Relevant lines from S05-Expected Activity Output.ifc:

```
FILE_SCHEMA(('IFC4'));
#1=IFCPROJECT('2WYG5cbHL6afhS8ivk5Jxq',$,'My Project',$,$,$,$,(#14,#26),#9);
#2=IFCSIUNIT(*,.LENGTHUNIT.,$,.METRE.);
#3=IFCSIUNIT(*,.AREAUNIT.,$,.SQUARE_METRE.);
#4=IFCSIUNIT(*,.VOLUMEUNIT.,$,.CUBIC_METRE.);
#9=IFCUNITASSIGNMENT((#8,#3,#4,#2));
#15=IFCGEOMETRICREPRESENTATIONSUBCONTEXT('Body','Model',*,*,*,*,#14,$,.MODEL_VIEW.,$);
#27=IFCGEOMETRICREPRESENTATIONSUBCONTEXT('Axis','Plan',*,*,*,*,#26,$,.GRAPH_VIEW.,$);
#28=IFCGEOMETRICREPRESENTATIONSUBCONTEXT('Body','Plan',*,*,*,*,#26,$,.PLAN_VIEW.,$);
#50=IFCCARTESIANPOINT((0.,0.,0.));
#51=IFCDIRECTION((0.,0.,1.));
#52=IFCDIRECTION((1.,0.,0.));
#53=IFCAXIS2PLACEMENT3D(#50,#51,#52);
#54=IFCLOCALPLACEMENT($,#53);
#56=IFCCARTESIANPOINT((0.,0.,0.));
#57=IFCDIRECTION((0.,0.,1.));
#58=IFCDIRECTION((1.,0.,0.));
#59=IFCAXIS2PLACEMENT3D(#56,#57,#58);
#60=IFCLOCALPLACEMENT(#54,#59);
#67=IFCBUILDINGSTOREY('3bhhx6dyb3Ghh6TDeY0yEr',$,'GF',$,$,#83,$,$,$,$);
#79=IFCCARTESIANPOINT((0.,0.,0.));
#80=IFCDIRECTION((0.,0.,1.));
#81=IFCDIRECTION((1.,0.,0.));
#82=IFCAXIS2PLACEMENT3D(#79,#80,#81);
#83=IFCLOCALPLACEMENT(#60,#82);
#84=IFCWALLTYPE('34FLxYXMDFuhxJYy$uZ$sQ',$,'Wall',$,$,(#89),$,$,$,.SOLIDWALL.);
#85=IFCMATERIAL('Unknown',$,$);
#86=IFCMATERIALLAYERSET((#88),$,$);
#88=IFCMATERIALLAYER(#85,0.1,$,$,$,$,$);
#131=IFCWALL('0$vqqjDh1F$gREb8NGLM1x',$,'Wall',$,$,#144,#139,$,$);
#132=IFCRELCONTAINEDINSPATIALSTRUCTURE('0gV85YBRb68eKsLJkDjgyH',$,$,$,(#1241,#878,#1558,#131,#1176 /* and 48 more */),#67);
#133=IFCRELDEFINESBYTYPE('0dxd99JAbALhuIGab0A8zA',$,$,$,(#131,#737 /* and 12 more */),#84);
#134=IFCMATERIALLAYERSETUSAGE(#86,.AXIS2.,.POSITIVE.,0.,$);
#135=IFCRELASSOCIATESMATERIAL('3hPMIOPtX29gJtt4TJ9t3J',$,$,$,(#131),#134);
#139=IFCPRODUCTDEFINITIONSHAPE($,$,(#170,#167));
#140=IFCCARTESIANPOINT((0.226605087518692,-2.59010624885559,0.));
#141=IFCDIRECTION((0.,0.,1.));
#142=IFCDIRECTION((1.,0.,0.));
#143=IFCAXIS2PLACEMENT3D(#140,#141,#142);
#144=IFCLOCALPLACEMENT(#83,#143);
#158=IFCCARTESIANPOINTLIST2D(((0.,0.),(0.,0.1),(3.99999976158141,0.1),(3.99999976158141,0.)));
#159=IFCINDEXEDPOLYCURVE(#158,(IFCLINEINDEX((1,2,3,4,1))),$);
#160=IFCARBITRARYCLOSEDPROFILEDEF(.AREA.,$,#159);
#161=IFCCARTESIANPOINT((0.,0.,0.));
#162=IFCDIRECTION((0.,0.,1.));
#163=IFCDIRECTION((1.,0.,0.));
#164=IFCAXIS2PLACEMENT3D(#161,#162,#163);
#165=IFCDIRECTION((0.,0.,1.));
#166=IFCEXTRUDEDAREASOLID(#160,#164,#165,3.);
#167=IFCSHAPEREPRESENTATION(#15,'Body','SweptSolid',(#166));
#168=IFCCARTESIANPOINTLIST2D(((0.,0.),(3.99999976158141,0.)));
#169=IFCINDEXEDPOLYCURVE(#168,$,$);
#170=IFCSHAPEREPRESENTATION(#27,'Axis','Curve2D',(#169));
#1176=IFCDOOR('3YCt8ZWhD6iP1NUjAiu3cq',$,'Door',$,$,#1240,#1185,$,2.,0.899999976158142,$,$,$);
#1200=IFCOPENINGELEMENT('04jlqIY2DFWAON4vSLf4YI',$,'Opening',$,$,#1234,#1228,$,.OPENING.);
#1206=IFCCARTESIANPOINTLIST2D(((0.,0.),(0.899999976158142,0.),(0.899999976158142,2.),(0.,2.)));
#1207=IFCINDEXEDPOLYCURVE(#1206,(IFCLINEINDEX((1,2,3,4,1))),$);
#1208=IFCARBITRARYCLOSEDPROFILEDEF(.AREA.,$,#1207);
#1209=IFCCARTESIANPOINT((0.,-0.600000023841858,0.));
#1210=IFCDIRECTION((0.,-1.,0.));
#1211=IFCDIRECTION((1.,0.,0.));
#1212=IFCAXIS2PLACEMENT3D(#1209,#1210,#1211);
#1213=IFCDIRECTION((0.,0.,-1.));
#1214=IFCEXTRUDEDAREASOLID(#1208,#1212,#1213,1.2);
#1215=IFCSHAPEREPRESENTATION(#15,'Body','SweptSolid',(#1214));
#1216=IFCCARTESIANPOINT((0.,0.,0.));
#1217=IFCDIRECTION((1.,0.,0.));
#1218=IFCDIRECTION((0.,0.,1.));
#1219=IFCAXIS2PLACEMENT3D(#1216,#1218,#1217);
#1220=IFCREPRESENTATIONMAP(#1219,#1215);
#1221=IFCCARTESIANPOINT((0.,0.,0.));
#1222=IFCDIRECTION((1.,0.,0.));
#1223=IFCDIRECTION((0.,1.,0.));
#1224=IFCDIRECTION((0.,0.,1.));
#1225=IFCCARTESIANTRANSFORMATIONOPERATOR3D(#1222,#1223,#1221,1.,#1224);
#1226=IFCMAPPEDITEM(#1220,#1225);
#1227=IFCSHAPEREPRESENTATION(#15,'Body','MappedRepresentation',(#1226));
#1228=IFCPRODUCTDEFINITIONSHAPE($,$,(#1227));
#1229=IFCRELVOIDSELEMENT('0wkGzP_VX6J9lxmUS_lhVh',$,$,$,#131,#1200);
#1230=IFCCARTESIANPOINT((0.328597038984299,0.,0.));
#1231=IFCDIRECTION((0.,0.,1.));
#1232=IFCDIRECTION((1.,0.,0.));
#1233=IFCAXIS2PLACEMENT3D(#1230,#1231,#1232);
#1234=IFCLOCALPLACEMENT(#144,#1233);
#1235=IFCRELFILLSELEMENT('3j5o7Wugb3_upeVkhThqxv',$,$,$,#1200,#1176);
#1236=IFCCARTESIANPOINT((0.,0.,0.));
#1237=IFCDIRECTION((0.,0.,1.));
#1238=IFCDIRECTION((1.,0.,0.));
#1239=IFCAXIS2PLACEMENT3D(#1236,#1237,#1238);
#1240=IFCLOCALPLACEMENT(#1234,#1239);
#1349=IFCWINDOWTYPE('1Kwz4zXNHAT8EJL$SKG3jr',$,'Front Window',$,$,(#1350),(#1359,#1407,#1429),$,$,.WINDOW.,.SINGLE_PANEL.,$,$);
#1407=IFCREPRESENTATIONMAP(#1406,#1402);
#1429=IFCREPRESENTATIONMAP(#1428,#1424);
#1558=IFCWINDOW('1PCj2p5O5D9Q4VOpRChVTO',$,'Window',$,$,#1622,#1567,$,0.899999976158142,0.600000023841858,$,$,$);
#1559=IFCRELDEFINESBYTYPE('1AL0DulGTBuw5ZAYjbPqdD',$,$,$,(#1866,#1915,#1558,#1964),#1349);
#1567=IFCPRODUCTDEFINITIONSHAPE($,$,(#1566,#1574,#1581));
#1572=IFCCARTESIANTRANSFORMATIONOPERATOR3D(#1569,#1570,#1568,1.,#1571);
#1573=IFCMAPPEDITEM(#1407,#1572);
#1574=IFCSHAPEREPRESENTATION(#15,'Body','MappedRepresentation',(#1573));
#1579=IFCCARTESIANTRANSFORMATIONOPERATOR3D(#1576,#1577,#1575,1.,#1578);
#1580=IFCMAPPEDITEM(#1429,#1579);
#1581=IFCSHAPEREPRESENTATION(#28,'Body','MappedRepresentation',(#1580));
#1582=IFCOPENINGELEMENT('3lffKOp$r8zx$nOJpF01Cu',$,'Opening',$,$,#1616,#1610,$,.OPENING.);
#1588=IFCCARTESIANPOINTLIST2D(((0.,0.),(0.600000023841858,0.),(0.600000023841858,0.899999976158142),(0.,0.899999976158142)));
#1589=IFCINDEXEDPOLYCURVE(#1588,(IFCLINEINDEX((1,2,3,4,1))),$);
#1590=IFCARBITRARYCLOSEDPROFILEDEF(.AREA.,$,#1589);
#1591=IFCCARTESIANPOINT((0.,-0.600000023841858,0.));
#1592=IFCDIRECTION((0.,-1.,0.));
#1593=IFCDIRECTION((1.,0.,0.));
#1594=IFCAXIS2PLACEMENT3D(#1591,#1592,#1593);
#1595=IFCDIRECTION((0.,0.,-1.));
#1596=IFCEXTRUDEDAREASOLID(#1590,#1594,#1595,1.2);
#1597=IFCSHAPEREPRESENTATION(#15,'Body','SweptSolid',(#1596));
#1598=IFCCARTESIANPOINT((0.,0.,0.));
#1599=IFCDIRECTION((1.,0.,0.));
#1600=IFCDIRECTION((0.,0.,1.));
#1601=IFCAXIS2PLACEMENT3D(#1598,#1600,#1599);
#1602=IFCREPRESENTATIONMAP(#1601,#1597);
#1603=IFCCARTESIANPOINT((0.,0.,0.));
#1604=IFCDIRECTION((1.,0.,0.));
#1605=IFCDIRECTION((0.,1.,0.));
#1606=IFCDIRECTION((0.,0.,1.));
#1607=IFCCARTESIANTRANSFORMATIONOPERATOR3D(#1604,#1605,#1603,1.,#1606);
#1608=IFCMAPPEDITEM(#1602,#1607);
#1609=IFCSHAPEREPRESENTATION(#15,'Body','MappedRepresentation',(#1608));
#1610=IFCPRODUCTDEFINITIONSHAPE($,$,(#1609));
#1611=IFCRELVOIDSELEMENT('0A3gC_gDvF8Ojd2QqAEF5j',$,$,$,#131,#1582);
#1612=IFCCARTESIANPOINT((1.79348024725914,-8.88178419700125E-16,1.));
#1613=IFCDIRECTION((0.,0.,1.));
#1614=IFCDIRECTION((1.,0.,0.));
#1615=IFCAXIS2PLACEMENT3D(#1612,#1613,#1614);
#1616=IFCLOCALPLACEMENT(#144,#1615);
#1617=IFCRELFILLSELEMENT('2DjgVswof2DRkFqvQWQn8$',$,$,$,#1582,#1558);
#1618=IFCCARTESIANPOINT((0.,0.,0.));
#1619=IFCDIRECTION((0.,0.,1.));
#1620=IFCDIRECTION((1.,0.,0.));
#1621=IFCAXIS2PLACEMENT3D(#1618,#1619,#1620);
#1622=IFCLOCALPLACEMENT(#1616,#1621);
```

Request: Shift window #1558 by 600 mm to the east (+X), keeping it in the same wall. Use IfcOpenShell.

```python
import ifcopenshell
import ifcopenshell.api.geometry
import ifcopenshell.util.placement

model = ifcopenshell.open("S05-Expected Activity Output.ifc")

window = model.by_guid("1PCj2p5O5D9Q4VOpRChVTO")
opening = window.FillsVoids[0].RelatingOpeningElement
wall = opening.VoidsElements[0].RelatingBuildingElement

wall_matrix = ifcopenshell.util.placement.get_local_placement(wall.ObjectPlacement)
shift = wall_matrix[:3, 0] * 0.6
before = ifcopenshell.util.placement.get_local_placement(window.ObjectPlacement)[:3, 3].copy()

# The window is placed relative to its opening, so it follows when the opening moves.
matrix = ifcopenshell.util.placement.get_local_placement(opening.ObjectPlacement)
matrix[:3, 3] += shift
ifcopenshell.api.geometry.edit_object_placement(
    model, product=opening, matrix=matrix, is_si=False, should_transform_children=True
)

after = ifcopenshell.util.placement.get_local_placement(window.ObjectPlacement)[:3, 3]
print("window moved by", (after - before).round(3) + 0.0)

model.write("S05-Expected Activity Output_updated.ifc")
```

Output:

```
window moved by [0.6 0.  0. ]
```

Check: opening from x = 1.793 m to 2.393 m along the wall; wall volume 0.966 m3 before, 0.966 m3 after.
